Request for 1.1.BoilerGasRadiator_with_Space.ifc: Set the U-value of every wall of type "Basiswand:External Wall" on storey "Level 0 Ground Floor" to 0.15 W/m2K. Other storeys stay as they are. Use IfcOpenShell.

First a look at what the model holds.

```python
import ifcopenshell
import ifcopenshell.util.element

model = ifcopenshell.open("1.1.BoilerGasRadiator_with_Space.ifc")
print(model.schema)
storey = next(s for s in model.by_type("IfcBuildingStorey") if s.Name == "Level 0 Ground Floor")
walls = [e for e in ifcopenshell.util.element.get_decomposition(storey) if e.is_a("IfcWall")]
seen = {}
for e in walls:
    element_type = ifcopenshell.util.element.get_type(e)
    key = (element_type.Name if element_type != e and element_type else None, ifcopenshell.util.element.get_pset(e, "Pset_WallCommon", "ThermalTransmittance"))
    seen[key] = seen.get(key, 0) + 1
for (name, value), count in sorted(seen.items(), key=str):
    print(count, "x", name, "|", value)
```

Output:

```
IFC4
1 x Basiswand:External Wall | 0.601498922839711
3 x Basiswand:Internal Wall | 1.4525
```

```python
import ifcopenshell
import ifcopenshell.api.pset
import ifcopenshell.util.element

model = ifcopenshell.open("1.1.BoilerGasRadiator_with_Space.ifc")

storey = next(s for s in model.by_type("IfcBuildingStorey") if s.Name == "Level 0 Ground Floor")
walls = [e for e in ifcopenshell.util.element.get_decomposition(storey) if e.is_a("IfcWall")]

count = 0
for e in walls:
    element_type = ifcopenshell.util.element.get_type(e)
    if element_type in (None, e) or element_type.Name != "Basiswand:External Wall":
        continue
    # add_pset returns the element's existing set when there is one.
    pset = ifcopenshell.api.pset.add_pset(model, product=e, name="Pset_WallCommon")
    ifcopenshell.api.pset.edit_pset(model, pset=pset, properties={"ThermalTransmittance": 0.15})
    count += 1

print(count, "walls updated")

model.write("1.1.BoilerGasRadiator_with_Space_updated.ifc")
```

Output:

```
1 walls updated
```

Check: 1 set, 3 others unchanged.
